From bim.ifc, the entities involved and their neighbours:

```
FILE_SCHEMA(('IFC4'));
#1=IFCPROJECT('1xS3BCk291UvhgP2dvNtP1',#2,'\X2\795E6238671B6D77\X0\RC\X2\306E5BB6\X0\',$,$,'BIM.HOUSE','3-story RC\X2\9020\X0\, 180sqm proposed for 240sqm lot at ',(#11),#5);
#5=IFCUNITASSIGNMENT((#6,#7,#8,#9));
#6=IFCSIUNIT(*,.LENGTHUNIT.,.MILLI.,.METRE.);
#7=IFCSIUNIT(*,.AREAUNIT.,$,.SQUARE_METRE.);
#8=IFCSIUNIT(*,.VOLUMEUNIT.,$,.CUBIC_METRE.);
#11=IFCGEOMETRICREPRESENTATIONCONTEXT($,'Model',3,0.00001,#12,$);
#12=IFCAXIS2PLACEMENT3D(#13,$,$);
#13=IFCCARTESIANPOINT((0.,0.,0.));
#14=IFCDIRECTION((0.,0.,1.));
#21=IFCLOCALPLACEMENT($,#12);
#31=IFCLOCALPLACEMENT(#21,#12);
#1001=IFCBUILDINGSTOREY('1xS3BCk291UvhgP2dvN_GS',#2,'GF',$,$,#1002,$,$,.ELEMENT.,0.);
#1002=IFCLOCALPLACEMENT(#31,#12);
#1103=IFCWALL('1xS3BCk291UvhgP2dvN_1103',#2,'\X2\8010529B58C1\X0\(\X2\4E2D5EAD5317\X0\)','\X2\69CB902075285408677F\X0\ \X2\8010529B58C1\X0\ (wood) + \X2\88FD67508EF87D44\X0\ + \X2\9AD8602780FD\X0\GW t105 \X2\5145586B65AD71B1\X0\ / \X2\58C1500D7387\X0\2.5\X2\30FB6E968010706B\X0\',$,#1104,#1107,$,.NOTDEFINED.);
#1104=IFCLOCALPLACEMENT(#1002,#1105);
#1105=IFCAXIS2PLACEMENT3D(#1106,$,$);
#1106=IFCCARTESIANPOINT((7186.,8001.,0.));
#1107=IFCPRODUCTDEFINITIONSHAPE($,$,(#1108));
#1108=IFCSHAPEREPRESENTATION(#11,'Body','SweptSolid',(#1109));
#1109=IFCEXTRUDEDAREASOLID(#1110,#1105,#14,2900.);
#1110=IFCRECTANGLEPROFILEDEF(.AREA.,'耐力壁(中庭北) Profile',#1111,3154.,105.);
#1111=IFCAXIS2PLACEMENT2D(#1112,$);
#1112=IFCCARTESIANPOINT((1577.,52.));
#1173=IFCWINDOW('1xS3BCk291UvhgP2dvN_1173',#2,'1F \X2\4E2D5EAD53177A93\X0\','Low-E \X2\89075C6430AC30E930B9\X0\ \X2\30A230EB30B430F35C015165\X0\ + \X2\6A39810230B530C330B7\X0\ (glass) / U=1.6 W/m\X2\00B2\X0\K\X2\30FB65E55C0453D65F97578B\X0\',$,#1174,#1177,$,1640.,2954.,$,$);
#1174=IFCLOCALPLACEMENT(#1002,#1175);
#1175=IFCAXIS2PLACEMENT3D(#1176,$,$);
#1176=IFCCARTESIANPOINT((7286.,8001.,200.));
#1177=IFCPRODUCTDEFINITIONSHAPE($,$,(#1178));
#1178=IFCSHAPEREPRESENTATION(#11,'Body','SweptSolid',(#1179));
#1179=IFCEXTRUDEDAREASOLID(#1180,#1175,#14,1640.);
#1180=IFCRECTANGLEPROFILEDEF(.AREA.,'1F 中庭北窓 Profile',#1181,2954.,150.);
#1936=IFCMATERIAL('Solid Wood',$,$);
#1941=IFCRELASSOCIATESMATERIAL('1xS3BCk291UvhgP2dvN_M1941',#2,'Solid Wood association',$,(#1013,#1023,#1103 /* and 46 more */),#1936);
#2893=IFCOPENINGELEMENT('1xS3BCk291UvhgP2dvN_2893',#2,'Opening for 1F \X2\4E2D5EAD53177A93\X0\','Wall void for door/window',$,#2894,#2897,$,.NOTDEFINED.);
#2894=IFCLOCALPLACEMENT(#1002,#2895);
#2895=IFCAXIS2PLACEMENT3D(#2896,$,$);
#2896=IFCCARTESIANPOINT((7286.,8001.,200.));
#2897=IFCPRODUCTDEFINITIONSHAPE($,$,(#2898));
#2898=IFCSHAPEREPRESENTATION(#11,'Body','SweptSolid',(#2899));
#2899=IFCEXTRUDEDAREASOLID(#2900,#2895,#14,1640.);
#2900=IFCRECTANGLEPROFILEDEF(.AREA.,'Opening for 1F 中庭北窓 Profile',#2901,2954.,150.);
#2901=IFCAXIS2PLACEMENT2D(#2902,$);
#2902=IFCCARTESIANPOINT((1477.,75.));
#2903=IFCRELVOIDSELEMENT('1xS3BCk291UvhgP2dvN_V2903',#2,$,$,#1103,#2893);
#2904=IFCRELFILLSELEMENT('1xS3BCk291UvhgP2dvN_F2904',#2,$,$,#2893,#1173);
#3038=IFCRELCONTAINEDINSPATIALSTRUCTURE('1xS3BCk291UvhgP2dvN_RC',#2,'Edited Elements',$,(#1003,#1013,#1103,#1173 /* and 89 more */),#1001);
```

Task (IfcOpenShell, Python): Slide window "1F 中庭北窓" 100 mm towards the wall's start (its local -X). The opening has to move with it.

```python
import ifcopenshell
import ifcopenshell.api.geometry
import ifcopenshell.util.placement
import ifcopenshell.util.unit

model = ifcopenshell.open("bim.ifc")
unit_scale = ifcopenshell.util.unit.calculate_unit_scale(model)

window = model.by_id(1173)
opening = window.FillsVoids[0].RelatingOpeningElement
wall = opening.VoidsElements[0].RelatingBuildingElement

wall_matrix = ifcopenshell.util.placement.get_local_placement(wall.ObjectPlacement)
shift = wall_matrix[:3, 0] * -0.1 / unit_scale
before = ifcopenshell.util.placement.get_local_placement(window.ObjectPlacement)[:3, 3].copy()

# The window is not placed relative to its opening, so move both.
for product in (opening, window):
    matrix = ifcopenshell.util.placement.get_local_placement(product.ObjectPlacement)
    matrix[:3, 3] += shift
    ifcopenshell.api.geometry.edit_object_placement(model, product=product, matrix=matrix, is_si=False)

after = ifcopenshell.util.placement.get_local_placement(window.ObjectPlacement)[:3, 3]
print("window moved by", (after - before).round(3) + 0.0)

model.write("bim-out.ifc")
```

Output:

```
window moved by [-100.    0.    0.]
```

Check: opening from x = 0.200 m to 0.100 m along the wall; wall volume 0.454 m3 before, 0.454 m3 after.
